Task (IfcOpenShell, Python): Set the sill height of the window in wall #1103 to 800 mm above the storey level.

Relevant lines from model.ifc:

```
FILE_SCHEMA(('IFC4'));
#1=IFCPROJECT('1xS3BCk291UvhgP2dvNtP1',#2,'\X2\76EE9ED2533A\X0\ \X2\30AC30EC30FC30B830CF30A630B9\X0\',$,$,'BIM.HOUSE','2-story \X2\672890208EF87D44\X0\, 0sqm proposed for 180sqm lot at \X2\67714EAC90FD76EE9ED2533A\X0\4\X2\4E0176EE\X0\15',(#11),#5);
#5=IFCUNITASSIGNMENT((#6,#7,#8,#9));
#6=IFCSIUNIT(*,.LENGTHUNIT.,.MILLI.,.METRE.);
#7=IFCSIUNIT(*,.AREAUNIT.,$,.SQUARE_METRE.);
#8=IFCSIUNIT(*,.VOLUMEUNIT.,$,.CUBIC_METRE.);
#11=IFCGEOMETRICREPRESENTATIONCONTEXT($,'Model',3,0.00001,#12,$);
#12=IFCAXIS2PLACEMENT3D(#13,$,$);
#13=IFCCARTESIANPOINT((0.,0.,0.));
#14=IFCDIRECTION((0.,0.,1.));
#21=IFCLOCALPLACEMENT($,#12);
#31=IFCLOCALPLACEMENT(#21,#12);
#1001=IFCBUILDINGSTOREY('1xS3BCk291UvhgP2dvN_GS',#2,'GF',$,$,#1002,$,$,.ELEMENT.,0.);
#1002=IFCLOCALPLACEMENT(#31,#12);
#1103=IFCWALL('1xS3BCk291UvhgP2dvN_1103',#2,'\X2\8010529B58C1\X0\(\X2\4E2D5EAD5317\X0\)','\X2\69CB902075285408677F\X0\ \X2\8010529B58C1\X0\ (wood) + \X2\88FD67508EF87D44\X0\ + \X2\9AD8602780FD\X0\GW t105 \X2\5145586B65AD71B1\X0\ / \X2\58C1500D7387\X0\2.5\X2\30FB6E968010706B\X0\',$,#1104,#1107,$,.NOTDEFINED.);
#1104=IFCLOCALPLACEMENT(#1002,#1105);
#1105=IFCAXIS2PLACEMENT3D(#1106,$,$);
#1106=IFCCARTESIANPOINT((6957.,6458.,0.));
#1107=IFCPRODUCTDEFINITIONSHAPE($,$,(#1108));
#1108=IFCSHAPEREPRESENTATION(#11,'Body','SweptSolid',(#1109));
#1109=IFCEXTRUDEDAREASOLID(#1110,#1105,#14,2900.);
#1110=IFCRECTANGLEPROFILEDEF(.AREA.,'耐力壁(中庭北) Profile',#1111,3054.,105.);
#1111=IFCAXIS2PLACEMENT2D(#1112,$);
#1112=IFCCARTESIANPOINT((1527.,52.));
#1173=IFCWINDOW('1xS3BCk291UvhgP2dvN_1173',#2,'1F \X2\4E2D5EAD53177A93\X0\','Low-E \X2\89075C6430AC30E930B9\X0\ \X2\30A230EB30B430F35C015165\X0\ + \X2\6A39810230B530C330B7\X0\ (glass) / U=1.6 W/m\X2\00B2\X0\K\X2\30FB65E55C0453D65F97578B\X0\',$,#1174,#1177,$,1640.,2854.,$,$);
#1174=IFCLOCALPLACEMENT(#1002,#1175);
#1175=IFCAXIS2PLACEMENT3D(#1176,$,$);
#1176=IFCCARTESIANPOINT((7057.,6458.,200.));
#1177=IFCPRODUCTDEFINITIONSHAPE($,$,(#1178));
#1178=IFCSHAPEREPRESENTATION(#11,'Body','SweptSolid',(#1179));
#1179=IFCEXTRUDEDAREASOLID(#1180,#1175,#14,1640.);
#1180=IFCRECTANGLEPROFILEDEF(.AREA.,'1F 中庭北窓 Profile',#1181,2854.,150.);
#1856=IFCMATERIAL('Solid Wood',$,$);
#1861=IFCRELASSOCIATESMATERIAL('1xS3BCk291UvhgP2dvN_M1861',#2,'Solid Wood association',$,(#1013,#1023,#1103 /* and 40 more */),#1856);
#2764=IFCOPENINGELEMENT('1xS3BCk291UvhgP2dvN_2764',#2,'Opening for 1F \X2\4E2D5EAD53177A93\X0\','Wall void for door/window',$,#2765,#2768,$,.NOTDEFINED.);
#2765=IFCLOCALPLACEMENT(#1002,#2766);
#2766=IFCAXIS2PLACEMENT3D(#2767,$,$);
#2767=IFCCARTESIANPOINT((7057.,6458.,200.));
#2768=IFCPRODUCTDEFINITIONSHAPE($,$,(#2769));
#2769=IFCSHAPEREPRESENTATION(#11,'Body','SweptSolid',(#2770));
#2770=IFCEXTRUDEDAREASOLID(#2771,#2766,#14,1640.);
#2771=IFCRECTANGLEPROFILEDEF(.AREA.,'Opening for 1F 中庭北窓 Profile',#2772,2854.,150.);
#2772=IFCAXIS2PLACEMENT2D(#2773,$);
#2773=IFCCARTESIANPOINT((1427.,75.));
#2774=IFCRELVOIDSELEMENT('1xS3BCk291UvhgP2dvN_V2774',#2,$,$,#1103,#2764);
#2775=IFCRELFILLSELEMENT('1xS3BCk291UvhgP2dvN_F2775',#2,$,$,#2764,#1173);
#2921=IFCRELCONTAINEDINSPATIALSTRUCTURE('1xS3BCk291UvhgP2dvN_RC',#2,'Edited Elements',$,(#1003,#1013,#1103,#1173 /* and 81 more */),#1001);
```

```python
import numpy as np
import ifcopenshell
import ifcopenshell.api.geometry
import ifcopenshell.geom
import ifcopenshell.util.element
import ifcopenshell.util.placement
import ifcopenshell.util.shape
import ifcopenshell.util.unit

model = ifcopenshell.open("model.ifc")
unit_scale = ifcopenshell.util.unit.calculate_unit_scale(model)

window = model.by_guid("1xS3BCk291UvhgP2dvN_1173")
opening = window.FillsVoids[0].RelatingOpeningElement
storey = ifcopenshell.util.element.get_container(window, ifc_class="IfcBuildingStorey")
level = ifcopenshell.util.placement.get_local_placement(storey.ObjectPlacement)[2, 3]

# The opening's origin need not be at the sill, so measure its lowest point.
shape = ifcopenshell.geom.create_shape(ifcopenshell.geom.settings(), opening)
bottom = ifcopenshell.util.shape.get_shape_bottom_elevation(shape, shape.geometry) / unit_scale
dz = level + 800.0 - bottom

shift = np.array([0.0, 0.0, dz])
# The window is not placed relative to its opening, so move both.
for product in (opening, window):
    matrix = ifcopenshell.util.placement.get_local_placement(product.ObjectPlacement)
    matrix[:3, 3] += shift
    ifcopenshell.api.geometry.edit_object_placement(model, product=product, matrix=matrix, is_si=False)

print(f"moved by {dz * unit_scale:+.3f} m")

model.write("model_updated.ifc")
```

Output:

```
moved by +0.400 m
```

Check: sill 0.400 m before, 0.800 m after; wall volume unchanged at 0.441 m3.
